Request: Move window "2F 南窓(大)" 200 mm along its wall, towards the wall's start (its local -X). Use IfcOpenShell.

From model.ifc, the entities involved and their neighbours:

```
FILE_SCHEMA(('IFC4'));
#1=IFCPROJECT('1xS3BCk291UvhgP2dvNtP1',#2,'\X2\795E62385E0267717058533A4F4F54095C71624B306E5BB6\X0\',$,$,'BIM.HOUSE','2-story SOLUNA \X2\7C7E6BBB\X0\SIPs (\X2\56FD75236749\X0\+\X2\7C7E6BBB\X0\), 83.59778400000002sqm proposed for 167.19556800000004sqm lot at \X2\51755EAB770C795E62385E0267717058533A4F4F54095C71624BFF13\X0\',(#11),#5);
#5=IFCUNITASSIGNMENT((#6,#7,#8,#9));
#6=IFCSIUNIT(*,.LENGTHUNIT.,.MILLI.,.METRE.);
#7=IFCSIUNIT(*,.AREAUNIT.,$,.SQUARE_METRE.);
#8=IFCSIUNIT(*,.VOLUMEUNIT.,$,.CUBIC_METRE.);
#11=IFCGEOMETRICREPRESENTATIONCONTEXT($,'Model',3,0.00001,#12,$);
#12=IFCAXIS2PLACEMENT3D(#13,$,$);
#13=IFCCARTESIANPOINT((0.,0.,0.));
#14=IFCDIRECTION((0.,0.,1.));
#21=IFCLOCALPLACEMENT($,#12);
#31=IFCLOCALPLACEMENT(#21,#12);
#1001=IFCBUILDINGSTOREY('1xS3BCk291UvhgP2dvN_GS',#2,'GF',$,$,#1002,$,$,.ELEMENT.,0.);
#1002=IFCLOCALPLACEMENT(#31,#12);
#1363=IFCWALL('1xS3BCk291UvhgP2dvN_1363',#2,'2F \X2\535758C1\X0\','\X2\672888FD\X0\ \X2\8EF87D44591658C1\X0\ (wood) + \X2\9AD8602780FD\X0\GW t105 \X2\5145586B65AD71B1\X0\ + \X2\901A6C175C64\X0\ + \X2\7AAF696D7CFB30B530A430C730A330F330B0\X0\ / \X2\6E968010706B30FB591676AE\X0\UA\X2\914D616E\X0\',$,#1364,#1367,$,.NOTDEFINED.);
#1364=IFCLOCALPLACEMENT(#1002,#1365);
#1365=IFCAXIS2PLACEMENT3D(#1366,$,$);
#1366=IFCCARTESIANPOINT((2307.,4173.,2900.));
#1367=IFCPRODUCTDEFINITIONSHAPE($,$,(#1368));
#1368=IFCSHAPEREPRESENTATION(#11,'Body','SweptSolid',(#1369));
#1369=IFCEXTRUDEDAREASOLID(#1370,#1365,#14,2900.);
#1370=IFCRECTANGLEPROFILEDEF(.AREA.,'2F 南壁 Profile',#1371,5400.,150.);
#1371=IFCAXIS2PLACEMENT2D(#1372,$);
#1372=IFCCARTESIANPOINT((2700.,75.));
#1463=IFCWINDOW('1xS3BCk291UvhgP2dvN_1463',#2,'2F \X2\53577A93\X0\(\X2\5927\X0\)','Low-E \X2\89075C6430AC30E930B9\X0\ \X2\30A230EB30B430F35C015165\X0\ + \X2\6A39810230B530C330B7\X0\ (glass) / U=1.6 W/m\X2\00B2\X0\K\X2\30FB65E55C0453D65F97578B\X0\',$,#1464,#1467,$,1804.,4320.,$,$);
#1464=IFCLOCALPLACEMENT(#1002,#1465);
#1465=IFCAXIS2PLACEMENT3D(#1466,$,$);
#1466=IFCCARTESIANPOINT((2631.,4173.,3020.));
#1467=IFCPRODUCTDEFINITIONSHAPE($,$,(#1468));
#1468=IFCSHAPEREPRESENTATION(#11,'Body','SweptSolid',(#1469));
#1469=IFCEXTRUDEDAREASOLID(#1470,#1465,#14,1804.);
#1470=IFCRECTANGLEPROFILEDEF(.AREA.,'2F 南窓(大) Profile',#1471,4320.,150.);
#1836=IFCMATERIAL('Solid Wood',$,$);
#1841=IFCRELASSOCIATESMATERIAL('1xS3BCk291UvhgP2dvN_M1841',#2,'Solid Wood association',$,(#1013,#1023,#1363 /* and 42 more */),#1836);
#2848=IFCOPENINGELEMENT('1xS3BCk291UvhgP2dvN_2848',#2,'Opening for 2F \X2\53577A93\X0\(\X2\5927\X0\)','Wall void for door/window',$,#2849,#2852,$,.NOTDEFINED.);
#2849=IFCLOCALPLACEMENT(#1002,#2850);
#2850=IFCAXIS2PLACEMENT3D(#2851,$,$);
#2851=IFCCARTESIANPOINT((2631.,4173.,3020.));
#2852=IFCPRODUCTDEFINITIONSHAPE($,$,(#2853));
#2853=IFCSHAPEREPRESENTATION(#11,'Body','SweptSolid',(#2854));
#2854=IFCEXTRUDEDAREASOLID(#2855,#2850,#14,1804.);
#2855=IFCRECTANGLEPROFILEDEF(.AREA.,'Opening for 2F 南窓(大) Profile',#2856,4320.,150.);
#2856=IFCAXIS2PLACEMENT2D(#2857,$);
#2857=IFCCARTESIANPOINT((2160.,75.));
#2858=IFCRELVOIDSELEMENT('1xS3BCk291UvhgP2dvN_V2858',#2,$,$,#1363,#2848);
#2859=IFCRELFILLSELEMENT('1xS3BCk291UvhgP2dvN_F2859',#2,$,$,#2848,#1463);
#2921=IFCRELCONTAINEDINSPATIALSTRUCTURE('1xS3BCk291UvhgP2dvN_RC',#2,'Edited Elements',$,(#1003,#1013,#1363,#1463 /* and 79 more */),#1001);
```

```python
import ifcopenshell
import ifcopenshell.api.geometry
import ifcopenshell.util.placement

model = ifcopenshell.open("model.ifc")

window = model.by_guid("1xS3BCk291UvhgP2dvN_1463")
opening = window.FillsVoids[0].RelatingOpeningElement
wall = opening.VoidsElements[0].RelatingBuildingElement

wall_matrix = ifcopenshell.util.placement.get_local_placement(wall.ObjectPlacement)
shift = wall_matrix[:3, 0] * -200.0
before = ifcopenshell.util.placement.get_local_placement(window.ObjectPlacement)[:3, 3].copy()

# The window is not placed relative to its opening, so move both.
for product in (opening, window):
    matrix = ifcopenshell.util.placement.get_local_placement(product.ObjectPlacement)
    matrix[:3, 3] += shift
    ifcopenshell.api.geometry.edit_object_placement(model, product=product, matrix=matrix, is_si=False)

after = ifcopenshell.util.placement.get_local_placement(window.ObjectPlacement)[:3, 3]
print("window moved by", (after - before).round(3) + 0.0)

model.write("model_v2.ifc")
```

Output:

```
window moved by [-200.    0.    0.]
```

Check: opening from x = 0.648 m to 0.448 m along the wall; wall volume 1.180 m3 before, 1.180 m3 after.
